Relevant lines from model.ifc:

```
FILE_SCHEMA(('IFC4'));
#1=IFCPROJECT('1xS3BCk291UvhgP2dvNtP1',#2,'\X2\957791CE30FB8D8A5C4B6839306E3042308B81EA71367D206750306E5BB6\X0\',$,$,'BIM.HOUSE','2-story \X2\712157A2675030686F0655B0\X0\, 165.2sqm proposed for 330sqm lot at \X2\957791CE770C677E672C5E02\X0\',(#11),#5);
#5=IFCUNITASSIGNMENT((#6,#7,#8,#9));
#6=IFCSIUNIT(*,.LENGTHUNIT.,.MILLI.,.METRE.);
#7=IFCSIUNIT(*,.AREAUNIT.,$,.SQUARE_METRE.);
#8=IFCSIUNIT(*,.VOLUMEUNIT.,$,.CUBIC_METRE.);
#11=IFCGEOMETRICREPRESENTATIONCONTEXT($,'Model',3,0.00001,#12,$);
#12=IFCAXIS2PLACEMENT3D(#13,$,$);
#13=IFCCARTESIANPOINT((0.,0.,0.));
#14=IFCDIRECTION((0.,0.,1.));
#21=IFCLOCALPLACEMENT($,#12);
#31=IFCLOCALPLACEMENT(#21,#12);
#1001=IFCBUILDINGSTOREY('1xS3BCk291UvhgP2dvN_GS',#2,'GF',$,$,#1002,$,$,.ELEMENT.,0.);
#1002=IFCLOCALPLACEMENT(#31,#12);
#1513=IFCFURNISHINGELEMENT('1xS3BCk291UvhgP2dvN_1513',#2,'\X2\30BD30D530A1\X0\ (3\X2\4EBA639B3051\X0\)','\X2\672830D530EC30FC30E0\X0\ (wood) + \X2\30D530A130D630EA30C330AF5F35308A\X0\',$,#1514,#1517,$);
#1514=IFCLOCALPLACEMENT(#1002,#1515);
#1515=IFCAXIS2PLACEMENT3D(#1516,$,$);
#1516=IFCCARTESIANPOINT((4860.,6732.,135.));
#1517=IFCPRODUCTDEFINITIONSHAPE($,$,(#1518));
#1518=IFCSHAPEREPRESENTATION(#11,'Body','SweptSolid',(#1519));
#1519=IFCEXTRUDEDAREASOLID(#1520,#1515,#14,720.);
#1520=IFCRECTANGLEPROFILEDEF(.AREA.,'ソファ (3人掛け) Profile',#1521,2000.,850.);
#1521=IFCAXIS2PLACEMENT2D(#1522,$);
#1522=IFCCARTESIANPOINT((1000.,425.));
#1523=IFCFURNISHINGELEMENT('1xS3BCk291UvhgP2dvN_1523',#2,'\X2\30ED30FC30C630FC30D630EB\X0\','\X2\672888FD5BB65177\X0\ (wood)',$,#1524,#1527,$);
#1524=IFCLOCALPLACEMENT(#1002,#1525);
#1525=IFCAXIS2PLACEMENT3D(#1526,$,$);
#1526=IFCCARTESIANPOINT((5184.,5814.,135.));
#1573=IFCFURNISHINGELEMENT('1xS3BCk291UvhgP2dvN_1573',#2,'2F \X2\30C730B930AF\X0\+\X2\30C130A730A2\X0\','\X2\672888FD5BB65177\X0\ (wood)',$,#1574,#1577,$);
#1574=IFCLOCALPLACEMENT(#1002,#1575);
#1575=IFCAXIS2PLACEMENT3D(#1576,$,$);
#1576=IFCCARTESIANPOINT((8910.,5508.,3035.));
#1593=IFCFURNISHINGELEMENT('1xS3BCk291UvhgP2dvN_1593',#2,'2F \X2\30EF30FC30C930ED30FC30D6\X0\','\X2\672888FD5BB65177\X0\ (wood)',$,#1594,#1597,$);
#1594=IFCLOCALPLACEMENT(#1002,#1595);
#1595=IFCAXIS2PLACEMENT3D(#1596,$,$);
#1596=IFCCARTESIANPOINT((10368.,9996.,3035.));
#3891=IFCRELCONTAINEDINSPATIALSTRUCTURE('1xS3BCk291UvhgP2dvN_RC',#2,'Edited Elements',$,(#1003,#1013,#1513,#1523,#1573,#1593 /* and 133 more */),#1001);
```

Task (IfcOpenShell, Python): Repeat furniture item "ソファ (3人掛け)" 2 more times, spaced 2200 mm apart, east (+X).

```python
import numpy as np
import ifcopenshell
import ifcopenshell.api.geometry
import ifcopenshell.api.root
import ifcopenshell.util.element
import ifcopenshell.util.placement

model = ifcopenshell.open("model.ifc")


def reuse_history(source, copy):
    """copy_class also copies each property set's owner history, people and application; keep the originals."""
    for rel in copy.IsDefinedBy:
        if rel.is_a("IfcRelDefinesByProperties") and (history := rel.RelatingPropertyDefinition.OwnerHistory):
            rel.RelatingPropertyDefinition.OwnerHistory = source.OwnerHistory
            ifcopenshell.util.element.remove_deep2(model, history)


source = model.by_guid("1xS3BCk291UvhgP2dvN_1513")
base = ifcopenshell.util.placement.get_local_placement(source.ObjectPlacement)
step = np.array([1.0, 0.0, 0.0]) * 2200.0

for i in range(1, 3):
    copy = ifcopenshell.api.root.copy_class(model, product=source)
    copy.Representation = ifcopenshell.util.element.copy_deep(
        model, source.Representation, exclude=["IfcGeometricRepresentationContext", "IfcRepresentationMap"]
    )
    reuse_history(source, copy)
    matrix = base.copy()
    matrix[:3, 3] += i * step
    print("added at", matrix[:3, 3].round(3) + 0.0)
    ifcopenshell.api.geometry.edit_object_placement(model, product=copy, matrix=matrix, is_si=False)

model.write("model_rev.ifc")
```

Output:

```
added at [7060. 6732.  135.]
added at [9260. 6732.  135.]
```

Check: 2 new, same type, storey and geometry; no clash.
